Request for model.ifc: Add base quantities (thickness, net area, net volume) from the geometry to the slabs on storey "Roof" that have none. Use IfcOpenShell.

First a look at what the model holds.

```python
import ifcopenshell
import ifcopenshell.util.element
import ifcopenshell.util.unit

model = ifcopenshell.open("model.ifc")
print(model.schema)
for unit_type in ("LENGTHUNIT", "AREAUNIT", "VOLUMEUNIT"):
    print(unit_type, ifcopenshell.util.unit.calculate_unit_scale(model, unit_type))
storey = next(s for s in model.by_type("IfcBuildingStorey") if s.Name == "Roof")
slabs = [e for e in ifcopenshell.util.element.get_decomposition(storey) if e.is_a("IfcSlab")]
for e in sorted(slabs, key=lambda e: e.id()):
    print(e.id(), e.is_a(), e.Name, list(ifcopenshell.util.element.get_psets(e, qtos_only=True)), sep=" | ")
```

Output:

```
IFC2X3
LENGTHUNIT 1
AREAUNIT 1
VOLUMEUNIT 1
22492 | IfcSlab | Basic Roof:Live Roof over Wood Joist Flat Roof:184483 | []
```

```python
import ifcopenshell
import ifcopenshell.api.pset
import ifcopenshell.geom
import ifcopenshell.util.element
import ifcopenshell.util.shape
import ifcopenshell.util.unit

model = ifcopenshell.open("model.ifc")
unit_scale = ifcopenshell.util.unit.calculate_unit_scale(model)
area_scale = ifcopenshell.util.unit.calculate_unit_scale(model, "AREAUNIT")
volume_scale = ifcopenshell.util.unit.calculate_unit_scale(model, "VOLUMEUNIT")
settings = ifcopenshell.geom.settings()

storey = next(s for s in model.by_type("IfcBuildingStorey") if s.Name == "Roof")
slabs = [e for e in ifcopenshell.util.element.get_decomposition(storey) if e.is_a("IfcSlab")]

for e in sorted(slabs, key=lambda e: e.id()):
    if ifcopenshell.util.element.get_psets(e, qtos_only=True, should_inherit=False):
        continue
    # Geometry comes back in metres, in the element's own axes.
    shape = ifcopenshell.geom.create_shape(settings, e)
    values = {
        "Width": ifcopenshell.util.shape.get_z(shape.geometry) / unit_scale,
        "NetArea": ifcopenshell.util.shape.get_footprint_area(shape.geometry) / area_scale,
        "NetVolume": ifcopenshell.util.shape.get_volume(shape.geometry) / volume_scale,
    }
    qto = ifcopenshell.api.pset.add_qto(model, product=e, name="BaseQuantities")
    ifcopenshell.api.pset.edit_qto(model, qto=qto, properties=values)
    print(e.id(), {k: round(v, 3) for k, v in values.items()})

model.write("model_v2.ifc")
```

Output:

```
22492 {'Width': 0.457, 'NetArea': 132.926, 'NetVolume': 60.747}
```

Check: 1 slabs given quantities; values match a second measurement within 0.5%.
